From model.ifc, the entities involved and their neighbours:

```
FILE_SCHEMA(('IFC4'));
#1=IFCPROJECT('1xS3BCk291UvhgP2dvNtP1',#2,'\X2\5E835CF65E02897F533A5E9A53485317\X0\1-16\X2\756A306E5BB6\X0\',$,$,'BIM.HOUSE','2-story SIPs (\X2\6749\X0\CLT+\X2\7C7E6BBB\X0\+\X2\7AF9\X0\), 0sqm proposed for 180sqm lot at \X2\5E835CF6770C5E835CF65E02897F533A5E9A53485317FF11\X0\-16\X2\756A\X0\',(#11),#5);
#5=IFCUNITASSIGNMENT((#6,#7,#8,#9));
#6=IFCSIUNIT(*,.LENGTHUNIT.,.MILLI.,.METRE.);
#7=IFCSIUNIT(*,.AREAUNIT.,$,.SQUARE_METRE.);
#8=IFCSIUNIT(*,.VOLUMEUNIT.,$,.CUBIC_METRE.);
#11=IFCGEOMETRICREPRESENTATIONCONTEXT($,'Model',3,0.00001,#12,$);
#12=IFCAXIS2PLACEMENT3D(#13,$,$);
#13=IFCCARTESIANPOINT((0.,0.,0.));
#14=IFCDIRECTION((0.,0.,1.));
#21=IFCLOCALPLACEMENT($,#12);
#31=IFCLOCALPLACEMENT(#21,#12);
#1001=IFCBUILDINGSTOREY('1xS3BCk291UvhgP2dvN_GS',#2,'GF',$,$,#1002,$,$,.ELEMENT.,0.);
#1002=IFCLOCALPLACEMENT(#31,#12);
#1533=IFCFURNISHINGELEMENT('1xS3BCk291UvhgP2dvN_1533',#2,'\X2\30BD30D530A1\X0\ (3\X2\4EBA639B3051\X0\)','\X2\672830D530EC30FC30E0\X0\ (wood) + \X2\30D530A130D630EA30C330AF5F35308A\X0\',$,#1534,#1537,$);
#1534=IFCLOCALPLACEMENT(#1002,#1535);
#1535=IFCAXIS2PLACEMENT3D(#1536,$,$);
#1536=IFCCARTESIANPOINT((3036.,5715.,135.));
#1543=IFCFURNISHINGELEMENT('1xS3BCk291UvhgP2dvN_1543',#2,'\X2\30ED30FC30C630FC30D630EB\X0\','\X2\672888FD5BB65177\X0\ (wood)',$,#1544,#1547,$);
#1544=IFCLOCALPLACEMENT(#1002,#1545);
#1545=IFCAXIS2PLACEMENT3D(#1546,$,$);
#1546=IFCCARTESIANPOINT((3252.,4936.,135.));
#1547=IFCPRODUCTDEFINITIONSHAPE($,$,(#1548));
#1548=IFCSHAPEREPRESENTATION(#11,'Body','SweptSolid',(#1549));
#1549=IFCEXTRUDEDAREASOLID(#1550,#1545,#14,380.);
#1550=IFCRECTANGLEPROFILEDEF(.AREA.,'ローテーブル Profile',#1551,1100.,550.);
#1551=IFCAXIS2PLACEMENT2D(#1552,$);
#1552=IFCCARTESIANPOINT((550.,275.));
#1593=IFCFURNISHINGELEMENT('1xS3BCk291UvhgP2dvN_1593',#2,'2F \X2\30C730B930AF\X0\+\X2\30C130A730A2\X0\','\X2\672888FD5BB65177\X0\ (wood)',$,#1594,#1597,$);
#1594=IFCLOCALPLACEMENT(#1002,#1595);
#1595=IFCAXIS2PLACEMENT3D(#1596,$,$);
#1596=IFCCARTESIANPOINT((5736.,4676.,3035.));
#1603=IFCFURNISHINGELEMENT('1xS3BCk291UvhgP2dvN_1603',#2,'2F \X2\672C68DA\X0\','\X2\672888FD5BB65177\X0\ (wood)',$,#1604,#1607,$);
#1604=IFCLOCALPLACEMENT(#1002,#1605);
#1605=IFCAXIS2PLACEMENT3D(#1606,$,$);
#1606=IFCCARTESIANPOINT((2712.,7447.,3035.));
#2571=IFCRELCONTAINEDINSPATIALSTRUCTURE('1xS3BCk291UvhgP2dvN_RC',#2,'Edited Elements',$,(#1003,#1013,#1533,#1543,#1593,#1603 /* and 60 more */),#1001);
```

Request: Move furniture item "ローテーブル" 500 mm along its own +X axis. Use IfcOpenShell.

```python
import ifcopenshell
import ifcopenshell.api.geometry
import ifcopenshell.util.placement

model = ifcopenshell.open("model.ifc")

item = model.by_guid("1xS3BCk291UvhgP2dvN_1543")
matrix = ifcopenshell.util.placement.get_local_placement(item.ObjectPlacement)
matrix[:3, 3] += matrix[:3, 0] * 500.0
ifcopenshell.api.geometry.edit_object_placement(model, product=item, matrix=matrix, is_si=False)

print(ifcopenshell.util.placement.get_local_placement(item.ObjectPlacement).round(3) + 0.0)

model.write("model-out.ifc")
```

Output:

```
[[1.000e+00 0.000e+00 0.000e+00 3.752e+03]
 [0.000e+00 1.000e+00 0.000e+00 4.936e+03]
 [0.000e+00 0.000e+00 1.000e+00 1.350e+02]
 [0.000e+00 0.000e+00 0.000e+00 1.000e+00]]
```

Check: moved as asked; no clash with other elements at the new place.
